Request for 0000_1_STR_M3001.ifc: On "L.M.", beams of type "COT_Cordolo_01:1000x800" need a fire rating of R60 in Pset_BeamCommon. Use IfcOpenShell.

First a look at what the model holds.

```python
import ifcopenshell
import ifcopenshell.util.element

model = ifcopenshell.open("0000_1_STR_M3001.ifc")
print(model.schema)
storey = next(s for s in model.by_type("IfcBuildingStorey") if s.Name == "L.M.")
beams = [e for e in ifcopenshell.util.element.get_decomposition(storey) if e.is_a("IfcBeam")]
seen = {}
for e in beams:
    element_type = ifcopenshell.util.element.get_type(e)
    key = (element_type.Name if element_type != e and element_type else None, ifcopenshell.util.element.get_pset(e, "Pset_BeamCommon", "FireRating"))
    seen[key] = seen.get(key, 0) + 1
for (name, value), count in sorted(seen.items(), key=str):
    print(count, "x", name, "|", value)
```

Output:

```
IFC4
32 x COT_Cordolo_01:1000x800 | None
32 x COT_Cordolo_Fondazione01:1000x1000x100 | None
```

```python
import ifcopenshell
import ifcopenshell.api.pset
import ifcopenshell.util.element

model = ifcopenshell.open("0000_1_STR_M3001.ifc")

storey = next(s for s in model.by_type("IfcBuildingStorey") if s.Name == "L.M.")
beams = [e for e in ifcopenshell.util.element.get_decomposition(storey) if e.is_a("IfcBeam")]

count = 0
for e in beams:
    element_type = ifcopenshell.util.element.get_type(e)
    if element_type in (None, e) or element_type.Name != "COT_Cordolo_01:1000x800":
        continue
    # add_pset returns the element's existing set when there is one.
    pset = ifcopenshell.api.pset.add_pset(model, product=e, name="Pset_BeamCommon")
    ifcopenshell.api.pset.edit_pset(model, pset=pset, properties={"FireRating": "R60"})
    count += 1

print(count, "beams updated")

model.write("0000_1_STR_M3001_v2.ifc")
```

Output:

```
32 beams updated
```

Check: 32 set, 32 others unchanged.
